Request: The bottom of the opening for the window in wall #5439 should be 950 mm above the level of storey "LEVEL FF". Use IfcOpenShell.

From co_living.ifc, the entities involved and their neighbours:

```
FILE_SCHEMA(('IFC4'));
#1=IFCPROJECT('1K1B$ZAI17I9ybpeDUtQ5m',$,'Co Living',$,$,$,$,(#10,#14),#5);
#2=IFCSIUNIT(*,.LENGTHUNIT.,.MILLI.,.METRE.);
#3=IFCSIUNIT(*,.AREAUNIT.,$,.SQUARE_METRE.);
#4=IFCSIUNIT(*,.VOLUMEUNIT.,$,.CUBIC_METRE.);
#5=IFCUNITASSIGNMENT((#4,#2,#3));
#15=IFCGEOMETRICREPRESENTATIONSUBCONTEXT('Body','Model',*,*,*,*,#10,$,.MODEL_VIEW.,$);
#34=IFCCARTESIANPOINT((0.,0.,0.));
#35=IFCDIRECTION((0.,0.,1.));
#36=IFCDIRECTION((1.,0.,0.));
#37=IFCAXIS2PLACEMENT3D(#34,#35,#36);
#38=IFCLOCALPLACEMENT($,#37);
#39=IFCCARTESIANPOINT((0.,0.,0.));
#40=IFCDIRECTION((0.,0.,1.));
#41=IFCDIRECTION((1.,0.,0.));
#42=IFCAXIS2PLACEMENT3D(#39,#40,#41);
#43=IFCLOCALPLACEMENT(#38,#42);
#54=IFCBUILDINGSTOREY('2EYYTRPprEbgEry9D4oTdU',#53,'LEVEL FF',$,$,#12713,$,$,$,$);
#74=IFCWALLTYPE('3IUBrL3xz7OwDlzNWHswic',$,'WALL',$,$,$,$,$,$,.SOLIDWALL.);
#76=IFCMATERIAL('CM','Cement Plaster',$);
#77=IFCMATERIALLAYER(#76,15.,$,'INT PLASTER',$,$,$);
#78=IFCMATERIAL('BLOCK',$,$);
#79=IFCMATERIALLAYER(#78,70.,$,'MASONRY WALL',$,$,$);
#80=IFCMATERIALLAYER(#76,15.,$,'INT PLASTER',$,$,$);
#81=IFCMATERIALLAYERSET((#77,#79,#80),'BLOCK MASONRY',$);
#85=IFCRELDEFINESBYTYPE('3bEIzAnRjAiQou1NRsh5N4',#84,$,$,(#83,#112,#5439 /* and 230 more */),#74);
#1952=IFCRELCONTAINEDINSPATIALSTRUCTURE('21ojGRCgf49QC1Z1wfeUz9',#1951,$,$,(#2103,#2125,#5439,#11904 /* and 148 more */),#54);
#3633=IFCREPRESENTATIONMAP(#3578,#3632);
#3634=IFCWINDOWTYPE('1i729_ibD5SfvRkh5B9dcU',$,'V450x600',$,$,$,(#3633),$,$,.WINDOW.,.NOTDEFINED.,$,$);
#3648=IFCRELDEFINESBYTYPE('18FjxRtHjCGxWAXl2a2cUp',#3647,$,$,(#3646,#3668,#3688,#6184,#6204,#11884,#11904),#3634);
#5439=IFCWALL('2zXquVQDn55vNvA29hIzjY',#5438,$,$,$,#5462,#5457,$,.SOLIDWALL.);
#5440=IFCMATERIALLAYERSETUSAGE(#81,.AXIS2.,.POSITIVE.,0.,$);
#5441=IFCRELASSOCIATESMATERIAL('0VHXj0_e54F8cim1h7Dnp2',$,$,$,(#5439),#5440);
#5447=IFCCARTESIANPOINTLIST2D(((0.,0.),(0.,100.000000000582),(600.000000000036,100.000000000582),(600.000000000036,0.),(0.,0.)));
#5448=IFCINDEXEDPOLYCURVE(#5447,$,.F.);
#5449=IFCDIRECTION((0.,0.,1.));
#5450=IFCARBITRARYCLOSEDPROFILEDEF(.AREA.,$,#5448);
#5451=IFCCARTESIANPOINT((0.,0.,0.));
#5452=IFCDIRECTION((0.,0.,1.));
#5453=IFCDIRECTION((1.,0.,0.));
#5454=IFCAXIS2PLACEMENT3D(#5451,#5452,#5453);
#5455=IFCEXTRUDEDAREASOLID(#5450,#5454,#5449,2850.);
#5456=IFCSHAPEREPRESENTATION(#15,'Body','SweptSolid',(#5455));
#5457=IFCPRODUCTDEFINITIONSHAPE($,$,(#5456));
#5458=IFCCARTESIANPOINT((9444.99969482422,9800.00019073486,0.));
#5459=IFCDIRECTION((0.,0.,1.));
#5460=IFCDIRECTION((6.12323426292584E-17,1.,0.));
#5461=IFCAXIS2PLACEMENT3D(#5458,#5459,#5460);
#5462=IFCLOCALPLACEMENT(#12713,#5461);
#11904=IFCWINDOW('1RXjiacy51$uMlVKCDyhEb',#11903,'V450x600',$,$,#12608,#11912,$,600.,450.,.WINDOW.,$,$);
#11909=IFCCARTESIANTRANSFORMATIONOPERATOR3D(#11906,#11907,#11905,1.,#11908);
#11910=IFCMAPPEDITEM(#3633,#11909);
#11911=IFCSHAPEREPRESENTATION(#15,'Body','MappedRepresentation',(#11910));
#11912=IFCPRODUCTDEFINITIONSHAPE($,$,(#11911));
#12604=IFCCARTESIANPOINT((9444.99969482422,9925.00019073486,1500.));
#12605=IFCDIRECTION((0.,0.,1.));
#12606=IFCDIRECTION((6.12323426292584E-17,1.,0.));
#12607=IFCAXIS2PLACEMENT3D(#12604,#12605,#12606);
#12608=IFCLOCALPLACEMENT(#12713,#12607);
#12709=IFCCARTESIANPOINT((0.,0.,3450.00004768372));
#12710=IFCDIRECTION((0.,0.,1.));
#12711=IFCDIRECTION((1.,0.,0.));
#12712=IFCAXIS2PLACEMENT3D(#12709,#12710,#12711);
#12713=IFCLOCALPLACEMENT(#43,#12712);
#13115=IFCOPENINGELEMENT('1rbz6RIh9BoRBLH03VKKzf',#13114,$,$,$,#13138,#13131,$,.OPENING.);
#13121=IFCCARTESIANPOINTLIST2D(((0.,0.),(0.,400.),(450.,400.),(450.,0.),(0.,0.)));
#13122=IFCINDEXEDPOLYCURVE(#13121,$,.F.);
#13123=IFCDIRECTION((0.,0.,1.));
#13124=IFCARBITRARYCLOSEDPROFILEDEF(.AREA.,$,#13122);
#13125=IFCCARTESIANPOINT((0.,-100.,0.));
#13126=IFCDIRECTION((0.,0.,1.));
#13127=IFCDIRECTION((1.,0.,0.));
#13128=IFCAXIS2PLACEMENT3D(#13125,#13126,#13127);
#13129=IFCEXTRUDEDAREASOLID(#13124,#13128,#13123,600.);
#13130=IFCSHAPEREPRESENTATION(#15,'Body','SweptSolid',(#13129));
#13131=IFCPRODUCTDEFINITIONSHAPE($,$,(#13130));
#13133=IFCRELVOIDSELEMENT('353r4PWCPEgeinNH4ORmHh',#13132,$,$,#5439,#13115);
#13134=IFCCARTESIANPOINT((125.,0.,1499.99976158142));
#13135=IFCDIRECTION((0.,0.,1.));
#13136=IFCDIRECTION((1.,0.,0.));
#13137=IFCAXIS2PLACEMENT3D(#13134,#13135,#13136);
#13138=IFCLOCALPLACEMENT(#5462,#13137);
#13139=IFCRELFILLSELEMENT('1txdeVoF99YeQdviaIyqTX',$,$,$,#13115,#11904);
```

```python
import numpy as np
import ifcopenshell
import ifcopenshell.api.geometry
import ifcopenshell.geom
import ifcopenshell.util.element
import ifcopenshell.util.placement
import ifcopenshell.util.shape
import ifcopenshell.util.unit

model = ifcopenshell.open("co_living.ifc")
unit_scale = ifcopenshell.util.unit.calculate_unit_scale(model)

window = model.by_id(11904)
opening = window.FillsVoids[0].RelatingOpeningElement
storey = ifcopenshell.util.element.get_container(window, ifc_class="IfcBuildingStorey")
level = ifcopenshell.util.placement.get_local_placement(storey.ObjectPlacement)[2, 3]

# The opening's origin need not be at the sill, so measure its lowest point.
shape = ifcopenshell.geom.create_shape(ifcopenshell.geom.settings(), opening)
bottom = ifcopenshell.util.shape.get_shape_bottom_elevation(shape, shape.geometry) / unit_scale
dz = level + 0.95 / unit_scale - bottom

shift = np.array([0.0, 0.0, dz])
# The window is not placed relative to its opening, so move both.
for product in (opening, window):
    matrix = ifcopenshell.util.placement.get_local_placement(product.ObjectPlacement)
    matrix[:3, 3] += shift
    ifcopenshell.api.geometry.edit_object_placement(model, product=product, matrix=matrix, is_si=False)

print(f"moved by {dz * unit_scale:+.3f} m")

model.write("co_living_rev.ifc")
```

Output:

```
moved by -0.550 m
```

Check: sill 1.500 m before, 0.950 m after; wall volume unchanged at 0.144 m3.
